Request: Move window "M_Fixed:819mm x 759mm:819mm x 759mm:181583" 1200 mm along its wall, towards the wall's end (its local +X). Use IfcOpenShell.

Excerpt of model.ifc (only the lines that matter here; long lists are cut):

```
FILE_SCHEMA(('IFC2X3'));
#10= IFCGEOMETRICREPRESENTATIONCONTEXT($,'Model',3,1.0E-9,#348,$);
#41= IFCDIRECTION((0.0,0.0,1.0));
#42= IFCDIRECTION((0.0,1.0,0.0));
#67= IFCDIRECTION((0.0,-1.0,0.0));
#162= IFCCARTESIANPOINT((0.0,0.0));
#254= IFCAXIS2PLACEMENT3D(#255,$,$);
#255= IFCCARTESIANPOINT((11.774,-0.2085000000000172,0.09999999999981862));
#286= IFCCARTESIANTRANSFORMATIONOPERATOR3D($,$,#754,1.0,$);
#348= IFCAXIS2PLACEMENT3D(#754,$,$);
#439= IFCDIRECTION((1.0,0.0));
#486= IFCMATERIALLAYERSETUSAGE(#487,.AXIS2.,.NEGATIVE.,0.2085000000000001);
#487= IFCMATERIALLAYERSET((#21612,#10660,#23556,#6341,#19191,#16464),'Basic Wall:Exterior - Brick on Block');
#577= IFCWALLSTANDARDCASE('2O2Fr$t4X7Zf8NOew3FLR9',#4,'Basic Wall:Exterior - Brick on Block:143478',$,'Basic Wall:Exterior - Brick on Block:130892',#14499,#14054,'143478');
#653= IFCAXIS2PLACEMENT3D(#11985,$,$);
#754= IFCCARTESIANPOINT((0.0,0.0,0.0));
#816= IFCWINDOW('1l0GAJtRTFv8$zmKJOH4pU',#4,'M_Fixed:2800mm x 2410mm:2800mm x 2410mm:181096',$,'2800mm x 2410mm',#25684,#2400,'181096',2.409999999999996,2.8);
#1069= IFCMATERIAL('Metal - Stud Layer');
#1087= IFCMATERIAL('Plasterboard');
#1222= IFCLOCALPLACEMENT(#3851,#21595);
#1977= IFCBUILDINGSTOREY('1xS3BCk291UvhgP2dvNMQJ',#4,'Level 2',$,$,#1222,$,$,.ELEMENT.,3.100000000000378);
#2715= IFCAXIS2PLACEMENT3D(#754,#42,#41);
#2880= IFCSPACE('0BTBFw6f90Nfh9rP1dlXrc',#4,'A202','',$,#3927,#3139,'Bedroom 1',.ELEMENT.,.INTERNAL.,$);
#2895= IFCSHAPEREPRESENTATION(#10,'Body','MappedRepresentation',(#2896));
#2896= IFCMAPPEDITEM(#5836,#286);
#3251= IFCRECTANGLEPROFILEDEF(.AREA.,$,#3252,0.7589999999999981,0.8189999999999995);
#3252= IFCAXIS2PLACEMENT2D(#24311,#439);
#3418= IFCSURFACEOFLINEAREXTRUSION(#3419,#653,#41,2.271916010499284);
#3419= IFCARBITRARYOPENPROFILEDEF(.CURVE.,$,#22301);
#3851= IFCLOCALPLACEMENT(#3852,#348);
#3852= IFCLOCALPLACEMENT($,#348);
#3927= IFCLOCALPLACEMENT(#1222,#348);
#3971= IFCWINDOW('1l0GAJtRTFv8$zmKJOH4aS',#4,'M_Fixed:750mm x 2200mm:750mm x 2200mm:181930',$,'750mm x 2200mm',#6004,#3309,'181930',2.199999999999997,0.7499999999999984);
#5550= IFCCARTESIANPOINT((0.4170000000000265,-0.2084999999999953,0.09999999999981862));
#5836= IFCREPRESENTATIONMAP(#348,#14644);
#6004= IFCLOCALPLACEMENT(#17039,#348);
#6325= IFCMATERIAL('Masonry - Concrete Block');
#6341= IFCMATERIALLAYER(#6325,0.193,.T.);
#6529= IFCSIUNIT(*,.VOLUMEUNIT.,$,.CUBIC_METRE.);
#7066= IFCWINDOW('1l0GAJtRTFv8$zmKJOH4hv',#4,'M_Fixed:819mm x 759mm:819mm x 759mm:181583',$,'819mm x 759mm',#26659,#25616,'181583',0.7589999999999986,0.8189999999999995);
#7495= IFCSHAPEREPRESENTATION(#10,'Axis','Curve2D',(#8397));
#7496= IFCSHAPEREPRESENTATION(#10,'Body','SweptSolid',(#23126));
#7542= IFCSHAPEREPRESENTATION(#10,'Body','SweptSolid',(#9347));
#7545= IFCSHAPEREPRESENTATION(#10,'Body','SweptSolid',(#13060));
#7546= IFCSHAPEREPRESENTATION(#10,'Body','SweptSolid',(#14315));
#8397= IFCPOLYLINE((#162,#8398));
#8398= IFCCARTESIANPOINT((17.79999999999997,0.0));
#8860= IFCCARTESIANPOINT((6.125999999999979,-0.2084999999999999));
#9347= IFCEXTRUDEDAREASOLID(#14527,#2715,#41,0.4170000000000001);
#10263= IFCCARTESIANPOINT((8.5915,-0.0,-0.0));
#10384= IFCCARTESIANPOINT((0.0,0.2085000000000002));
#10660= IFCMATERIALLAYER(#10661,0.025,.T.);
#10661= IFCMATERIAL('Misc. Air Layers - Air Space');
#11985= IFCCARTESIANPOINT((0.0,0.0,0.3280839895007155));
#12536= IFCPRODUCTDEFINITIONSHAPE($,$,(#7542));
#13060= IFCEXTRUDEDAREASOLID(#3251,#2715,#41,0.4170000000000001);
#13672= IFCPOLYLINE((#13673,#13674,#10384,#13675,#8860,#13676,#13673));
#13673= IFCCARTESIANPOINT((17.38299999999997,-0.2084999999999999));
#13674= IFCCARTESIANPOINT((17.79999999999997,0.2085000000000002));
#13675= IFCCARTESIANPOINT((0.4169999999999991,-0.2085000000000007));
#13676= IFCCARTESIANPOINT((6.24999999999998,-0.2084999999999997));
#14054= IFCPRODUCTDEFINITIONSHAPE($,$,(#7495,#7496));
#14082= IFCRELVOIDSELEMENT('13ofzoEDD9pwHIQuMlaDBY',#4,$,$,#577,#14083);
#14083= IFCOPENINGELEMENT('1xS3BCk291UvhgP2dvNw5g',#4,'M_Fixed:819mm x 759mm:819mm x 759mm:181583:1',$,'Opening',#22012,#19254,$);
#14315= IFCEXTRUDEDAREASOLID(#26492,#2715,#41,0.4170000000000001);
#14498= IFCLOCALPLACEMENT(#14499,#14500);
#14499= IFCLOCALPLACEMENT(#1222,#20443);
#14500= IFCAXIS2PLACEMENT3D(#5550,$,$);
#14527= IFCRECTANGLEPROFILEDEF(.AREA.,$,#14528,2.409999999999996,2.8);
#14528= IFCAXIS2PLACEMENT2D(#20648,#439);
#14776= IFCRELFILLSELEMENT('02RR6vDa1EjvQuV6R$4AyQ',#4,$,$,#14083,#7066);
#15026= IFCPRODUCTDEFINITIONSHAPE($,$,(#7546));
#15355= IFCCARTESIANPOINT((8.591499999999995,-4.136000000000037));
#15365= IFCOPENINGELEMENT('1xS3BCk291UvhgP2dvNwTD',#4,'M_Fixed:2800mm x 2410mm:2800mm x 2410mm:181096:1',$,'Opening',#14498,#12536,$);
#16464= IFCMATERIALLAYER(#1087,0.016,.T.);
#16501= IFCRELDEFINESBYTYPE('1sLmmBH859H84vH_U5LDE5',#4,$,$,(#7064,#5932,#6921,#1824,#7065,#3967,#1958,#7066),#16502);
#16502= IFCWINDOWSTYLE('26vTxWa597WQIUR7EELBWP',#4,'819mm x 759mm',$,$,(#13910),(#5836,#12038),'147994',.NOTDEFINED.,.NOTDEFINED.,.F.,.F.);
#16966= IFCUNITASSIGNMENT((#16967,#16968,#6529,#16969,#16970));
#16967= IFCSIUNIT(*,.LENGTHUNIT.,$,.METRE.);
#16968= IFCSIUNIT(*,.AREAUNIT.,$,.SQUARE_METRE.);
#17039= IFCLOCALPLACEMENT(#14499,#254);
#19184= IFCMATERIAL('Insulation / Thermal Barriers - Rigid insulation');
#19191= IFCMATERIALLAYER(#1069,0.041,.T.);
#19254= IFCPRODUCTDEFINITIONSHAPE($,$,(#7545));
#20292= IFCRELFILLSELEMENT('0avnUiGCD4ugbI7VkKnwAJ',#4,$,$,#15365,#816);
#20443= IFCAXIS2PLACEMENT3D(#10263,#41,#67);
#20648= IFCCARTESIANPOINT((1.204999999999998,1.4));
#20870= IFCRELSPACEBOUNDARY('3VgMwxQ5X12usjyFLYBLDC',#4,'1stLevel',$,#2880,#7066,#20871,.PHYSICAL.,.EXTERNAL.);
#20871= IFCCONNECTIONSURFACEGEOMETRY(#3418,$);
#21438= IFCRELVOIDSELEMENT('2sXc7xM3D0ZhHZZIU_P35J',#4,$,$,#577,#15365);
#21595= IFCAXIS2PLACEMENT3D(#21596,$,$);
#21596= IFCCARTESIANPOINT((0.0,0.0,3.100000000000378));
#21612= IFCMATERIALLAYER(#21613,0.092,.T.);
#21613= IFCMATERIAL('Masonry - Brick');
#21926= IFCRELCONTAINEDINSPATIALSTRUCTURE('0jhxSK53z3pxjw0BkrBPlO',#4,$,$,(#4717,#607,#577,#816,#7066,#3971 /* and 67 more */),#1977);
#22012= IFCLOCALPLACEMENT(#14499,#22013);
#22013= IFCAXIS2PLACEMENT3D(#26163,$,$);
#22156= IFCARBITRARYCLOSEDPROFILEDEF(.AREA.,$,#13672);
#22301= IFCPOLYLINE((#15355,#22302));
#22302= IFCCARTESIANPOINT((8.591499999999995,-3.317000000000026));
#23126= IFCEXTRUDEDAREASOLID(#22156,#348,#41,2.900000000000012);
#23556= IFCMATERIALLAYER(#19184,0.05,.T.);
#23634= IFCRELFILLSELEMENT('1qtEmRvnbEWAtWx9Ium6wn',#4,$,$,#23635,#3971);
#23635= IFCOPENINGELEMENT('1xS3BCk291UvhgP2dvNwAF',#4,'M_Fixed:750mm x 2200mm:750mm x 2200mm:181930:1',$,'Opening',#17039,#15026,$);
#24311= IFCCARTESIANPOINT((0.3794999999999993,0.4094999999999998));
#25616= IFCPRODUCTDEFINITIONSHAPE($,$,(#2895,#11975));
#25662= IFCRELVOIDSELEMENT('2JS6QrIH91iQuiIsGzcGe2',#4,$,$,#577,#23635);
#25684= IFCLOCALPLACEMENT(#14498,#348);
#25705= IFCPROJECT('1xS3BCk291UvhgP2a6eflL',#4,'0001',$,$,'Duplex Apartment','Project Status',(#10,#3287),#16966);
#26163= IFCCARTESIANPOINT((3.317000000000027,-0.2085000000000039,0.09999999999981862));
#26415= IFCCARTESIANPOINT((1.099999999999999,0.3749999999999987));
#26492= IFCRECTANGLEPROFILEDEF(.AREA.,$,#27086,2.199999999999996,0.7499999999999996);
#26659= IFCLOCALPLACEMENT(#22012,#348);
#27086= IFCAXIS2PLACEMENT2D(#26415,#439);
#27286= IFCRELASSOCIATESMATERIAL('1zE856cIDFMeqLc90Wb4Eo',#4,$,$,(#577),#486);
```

```python
import numpy as np
import ifcopenshell
import ifcopenshell.api.geometry
import ifcopenshell.util.placement

model = ifcopenshell.open("model.ifc")

window = model.by_guid("1l0GAJtRTFv8$zmKJOH4hv")
opening = window.FillsVoids[0].RelatingOpeningElement
wall = opening.VoidsElements[0].RelatingBuildingElement

wall_matrix = ifcopenshell.util.placement.get_local_placement(wall.ObjectPlacement)
shift = wall_matrix[:3, 0] * 1.2
before = ifcopenshell.util.placement.get_local_placement(window.ObjectPlacement)[:3, 3].copy()

# The window is placed relative to its opening, so it follows when the opening moves.
matrix = ifcopenshell.util.placement.get_local_placement(opening.ObjectPlacement)
matrix[:3, 3] += shift
ifcopenshell.api.geometry.edit_object_placement(
    model, product=opening, matrix=matrix, is_si=False, should_transform_children=True
)

# Space boundary surfaces are stored in each space's coordinates; move them too.
for rel in window.ProvidesBoundaries:
    if not rel.ConnectionGeometry:
        continue
    surface = rel.ConnectionGeometry.SurfaceOnRelatingElement
    space_matrix = ifcopenshell.util.placement.get_local_placement(rel.RelatingSpace.ObjectPlacement)
    point = np.array(surface.Position.Location.Coordinates) + space_matrix[:3, :3].T @ shift
    surface.Position = model.createIfcAxis2Placement3D(
        model.createIfcCartesianPoint(point.tolist()), surface.Position.Axis, surface.Position.RefDirection
    )

after = ifcopenshell.util.placement.get_local_placement(window.ObjectPlacement)[:3, 3]
print("window moved by", (after - before).round(3) + 0.0)

model.write("model_edited.ifc")
```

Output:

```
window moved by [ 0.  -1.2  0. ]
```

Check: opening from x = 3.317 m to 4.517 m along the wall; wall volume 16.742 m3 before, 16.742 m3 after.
